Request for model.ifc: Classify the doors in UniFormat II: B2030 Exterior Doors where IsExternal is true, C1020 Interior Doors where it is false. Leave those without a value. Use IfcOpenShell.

First a look at what the model holds.

```python
import ifcopenshell
import ifcopenshell.util.element

model = ifcopenshell.open("model.ifc")
print(model.schema)
print("classifications:", [c.Name for c in model.by_type("IfcClassification")])
values = [ifcopenshell.util.element.get_pset(e, "Pset_DoorCommon", "IsExternal") for e in model.by_type("IfcDoor")]
for value in (True, False, None):
    print("IsExternal", value, values.count(value))
```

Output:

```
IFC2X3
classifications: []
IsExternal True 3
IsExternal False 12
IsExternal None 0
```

```python
import ifcopenshell
import ifcopenshell.api.classification
import ifcopenshell.util.element

model = ifcopenshell.open("model.ifc")

# IFC2X3 requires Source and Edition and has no link from the project to the system.
system = model.create_entity("IfcClassification", Source="ASTM", Edition="E1557", Name="UniFormat II")

doors = model.by_type("IfcDoor")
external = {e: ifcopenshell.util.element.get_pset(e, "Pset_DoorCommon", "IsExternal") for e in doors}
for flag, code, name in ((True, "B2030", "Exterior Doors"), (False, "C1020", "Interior Doors")):
    products = [e for e in doors if external[e] is flag]
    ifcopenshell.api.classification.add_reference(
        model, products=products, classification=system, identification=code, name=name
    )
    print(code, len(products))

model.write("model_edited.ifc")
```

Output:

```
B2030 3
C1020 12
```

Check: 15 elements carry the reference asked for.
